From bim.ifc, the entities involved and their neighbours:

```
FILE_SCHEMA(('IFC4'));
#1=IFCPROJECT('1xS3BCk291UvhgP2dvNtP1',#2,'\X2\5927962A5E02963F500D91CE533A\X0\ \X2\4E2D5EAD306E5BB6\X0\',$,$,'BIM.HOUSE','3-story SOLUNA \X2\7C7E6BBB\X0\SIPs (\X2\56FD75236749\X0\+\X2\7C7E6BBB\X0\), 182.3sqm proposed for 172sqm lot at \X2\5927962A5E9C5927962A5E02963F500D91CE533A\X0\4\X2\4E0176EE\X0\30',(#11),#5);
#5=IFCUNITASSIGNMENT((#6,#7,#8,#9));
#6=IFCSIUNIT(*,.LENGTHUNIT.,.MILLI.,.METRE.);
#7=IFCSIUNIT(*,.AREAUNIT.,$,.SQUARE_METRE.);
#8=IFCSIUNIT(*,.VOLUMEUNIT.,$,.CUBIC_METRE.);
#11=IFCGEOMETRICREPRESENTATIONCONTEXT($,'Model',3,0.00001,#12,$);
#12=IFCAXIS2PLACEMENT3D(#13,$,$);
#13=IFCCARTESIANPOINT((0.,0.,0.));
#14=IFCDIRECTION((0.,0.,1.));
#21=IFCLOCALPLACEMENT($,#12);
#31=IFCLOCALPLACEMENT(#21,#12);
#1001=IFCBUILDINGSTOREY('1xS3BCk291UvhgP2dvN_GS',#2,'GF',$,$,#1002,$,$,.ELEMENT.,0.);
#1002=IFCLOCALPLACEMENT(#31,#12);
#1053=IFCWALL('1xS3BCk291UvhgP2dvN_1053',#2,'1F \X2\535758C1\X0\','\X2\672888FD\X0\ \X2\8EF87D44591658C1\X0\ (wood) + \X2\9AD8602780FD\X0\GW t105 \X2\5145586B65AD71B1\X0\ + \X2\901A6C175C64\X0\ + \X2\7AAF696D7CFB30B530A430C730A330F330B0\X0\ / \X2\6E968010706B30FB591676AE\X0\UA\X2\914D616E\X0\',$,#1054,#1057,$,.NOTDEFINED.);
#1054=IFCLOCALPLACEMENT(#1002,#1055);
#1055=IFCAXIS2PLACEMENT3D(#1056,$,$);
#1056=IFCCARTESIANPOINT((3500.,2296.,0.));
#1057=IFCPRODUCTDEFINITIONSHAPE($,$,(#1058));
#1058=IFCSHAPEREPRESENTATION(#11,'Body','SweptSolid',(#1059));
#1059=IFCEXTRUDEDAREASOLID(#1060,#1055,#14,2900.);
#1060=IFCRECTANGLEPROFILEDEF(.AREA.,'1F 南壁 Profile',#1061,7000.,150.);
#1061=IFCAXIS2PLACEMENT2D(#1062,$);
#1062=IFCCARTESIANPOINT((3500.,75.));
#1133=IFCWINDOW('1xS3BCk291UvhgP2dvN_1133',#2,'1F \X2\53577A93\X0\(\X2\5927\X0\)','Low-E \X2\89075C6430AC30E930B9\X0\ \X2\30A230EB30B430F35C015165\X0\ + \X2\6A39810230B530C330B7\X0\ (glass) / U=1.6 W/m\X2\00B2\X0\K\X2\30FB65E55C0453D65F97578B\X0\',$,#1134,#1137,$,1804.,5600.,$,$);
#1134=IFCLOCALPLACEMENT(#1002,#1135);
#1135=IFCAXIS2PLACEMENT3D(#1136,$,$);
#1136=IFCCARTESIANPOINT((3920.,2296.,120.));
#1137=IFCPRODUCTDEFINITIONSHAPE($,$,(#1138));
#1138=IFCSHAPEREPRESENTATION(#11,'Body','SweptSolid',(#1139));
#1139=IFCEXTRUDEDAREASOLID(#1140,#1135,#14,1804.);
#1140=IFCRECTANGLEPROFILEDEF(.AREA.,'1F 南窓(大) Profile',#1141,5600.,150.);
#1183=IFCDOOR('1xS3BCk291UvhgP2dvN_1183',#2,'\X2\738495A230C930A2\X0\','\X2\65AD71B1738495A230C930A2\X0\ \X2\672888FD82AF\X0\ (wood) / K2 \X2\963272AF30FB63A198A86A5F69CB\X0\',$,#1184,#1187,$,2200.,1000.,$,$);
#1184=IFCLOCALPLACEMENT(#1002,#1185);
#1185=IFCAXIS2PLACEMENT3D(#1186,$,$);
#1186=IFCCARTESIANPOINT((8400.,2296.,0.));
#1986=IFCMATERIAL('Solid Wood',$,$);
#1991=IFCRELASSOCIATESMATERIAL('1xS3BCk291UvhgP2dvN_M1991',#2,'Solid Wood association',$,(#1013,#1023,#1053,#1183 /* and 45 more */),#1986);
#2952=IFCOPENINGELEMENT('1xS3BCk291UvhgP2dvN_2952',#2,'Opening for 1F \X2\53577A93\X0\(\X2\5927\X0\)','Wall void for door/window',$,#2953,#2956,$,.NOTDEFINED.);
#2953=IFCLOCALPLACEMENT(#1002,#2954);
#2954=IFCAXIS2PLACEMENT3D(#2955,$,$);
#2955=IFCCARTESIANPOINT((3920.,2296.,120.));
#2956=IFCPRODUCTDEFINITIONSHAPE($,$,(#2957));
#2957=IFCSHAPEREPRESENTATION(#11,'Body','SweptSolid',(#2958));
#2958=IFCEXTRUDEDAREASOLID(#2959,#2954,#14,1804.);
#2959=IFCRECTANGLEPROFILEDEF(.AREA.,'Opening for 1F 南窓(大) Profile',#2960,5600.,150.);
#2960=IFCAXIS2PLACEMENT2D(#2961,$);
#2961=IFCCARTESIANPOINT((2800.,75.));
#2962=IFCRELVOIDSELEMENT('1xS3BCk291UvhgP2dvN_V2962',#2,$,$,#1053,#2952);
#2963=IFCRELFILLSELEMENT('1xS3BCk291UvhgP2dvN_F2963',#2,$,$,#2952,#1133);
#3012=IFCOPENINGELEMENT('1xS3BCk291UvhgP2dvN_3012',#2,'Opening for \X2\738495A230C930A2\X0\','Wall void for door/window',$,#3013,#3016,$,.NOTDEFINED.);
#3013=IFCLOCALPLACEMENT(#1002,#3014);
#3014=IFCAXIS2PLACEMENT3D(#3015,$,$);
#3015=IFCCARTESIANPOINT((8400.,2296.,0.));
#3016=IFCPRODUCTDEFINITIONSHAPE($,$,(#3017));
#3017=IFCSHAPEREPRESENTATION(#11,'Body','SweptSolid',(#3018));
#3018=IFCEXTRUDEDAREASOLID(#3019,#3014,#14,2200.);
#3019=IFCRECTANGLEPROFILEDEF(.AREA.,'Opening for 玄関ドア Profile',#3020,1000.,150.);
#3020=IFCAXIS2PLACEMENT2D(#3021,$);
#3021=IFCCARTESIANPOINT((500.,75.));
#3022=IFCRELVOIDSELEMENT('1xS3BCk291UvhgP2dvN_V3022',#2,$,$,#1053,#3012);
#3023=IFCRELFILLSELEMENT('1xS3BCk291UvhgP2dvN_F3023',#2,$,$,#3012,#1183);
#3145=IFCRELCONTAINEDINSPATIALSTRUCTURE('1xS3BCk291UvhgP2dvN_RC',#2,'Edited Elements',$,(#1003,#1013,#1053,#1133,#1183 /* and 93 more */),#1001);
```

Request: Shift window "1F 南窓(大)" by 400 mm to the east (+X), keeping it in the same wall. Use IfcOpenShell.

```python
import ifcopenshell
import ifcopenshell.api.geometry
import ifcopenshell.util.placement

model = ifcopenshell.open("bim.ifc")

window = model.by_guid("1xS3BCk291UvhgP2dvN_1133")
opening = window.FillsVoids[0].RelatingOpeningElement
wall = opening.VoidsElements[0].RelatingBuildingElement

wall_matrix = ifcopenshell.util.placement.get_local_placement(wall.ObjectPlacement)
shift = wall_matrix[:3, 0] * 400.0
before = ifcopenshell.util.placement.get_local_placement(window.ObjectPlacement)[:3, 3].copy()

# The window is not placed relative to its opening, so move both.
for product in (opening, window):
    matrix = ifcopenshell.util.placement.get_local_placement(product.ObjectPlacement)
    matrix[:3, 3] += shift
    ifcopenshell.api.geometry.edit_object_placement(model, product=product, matrix=matrix, is_si=False)

after = ifcopenshell.util.placement.get_local_placement(window.ObjectPlacement)[:3, 3]
print("window moved by", (after - before).round(3) + 0.0)

model.write("bim_v2.ifc")
```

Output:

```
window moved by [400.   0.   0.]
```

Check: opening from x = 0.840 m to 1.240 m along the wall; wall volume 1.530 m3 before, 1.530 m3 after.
